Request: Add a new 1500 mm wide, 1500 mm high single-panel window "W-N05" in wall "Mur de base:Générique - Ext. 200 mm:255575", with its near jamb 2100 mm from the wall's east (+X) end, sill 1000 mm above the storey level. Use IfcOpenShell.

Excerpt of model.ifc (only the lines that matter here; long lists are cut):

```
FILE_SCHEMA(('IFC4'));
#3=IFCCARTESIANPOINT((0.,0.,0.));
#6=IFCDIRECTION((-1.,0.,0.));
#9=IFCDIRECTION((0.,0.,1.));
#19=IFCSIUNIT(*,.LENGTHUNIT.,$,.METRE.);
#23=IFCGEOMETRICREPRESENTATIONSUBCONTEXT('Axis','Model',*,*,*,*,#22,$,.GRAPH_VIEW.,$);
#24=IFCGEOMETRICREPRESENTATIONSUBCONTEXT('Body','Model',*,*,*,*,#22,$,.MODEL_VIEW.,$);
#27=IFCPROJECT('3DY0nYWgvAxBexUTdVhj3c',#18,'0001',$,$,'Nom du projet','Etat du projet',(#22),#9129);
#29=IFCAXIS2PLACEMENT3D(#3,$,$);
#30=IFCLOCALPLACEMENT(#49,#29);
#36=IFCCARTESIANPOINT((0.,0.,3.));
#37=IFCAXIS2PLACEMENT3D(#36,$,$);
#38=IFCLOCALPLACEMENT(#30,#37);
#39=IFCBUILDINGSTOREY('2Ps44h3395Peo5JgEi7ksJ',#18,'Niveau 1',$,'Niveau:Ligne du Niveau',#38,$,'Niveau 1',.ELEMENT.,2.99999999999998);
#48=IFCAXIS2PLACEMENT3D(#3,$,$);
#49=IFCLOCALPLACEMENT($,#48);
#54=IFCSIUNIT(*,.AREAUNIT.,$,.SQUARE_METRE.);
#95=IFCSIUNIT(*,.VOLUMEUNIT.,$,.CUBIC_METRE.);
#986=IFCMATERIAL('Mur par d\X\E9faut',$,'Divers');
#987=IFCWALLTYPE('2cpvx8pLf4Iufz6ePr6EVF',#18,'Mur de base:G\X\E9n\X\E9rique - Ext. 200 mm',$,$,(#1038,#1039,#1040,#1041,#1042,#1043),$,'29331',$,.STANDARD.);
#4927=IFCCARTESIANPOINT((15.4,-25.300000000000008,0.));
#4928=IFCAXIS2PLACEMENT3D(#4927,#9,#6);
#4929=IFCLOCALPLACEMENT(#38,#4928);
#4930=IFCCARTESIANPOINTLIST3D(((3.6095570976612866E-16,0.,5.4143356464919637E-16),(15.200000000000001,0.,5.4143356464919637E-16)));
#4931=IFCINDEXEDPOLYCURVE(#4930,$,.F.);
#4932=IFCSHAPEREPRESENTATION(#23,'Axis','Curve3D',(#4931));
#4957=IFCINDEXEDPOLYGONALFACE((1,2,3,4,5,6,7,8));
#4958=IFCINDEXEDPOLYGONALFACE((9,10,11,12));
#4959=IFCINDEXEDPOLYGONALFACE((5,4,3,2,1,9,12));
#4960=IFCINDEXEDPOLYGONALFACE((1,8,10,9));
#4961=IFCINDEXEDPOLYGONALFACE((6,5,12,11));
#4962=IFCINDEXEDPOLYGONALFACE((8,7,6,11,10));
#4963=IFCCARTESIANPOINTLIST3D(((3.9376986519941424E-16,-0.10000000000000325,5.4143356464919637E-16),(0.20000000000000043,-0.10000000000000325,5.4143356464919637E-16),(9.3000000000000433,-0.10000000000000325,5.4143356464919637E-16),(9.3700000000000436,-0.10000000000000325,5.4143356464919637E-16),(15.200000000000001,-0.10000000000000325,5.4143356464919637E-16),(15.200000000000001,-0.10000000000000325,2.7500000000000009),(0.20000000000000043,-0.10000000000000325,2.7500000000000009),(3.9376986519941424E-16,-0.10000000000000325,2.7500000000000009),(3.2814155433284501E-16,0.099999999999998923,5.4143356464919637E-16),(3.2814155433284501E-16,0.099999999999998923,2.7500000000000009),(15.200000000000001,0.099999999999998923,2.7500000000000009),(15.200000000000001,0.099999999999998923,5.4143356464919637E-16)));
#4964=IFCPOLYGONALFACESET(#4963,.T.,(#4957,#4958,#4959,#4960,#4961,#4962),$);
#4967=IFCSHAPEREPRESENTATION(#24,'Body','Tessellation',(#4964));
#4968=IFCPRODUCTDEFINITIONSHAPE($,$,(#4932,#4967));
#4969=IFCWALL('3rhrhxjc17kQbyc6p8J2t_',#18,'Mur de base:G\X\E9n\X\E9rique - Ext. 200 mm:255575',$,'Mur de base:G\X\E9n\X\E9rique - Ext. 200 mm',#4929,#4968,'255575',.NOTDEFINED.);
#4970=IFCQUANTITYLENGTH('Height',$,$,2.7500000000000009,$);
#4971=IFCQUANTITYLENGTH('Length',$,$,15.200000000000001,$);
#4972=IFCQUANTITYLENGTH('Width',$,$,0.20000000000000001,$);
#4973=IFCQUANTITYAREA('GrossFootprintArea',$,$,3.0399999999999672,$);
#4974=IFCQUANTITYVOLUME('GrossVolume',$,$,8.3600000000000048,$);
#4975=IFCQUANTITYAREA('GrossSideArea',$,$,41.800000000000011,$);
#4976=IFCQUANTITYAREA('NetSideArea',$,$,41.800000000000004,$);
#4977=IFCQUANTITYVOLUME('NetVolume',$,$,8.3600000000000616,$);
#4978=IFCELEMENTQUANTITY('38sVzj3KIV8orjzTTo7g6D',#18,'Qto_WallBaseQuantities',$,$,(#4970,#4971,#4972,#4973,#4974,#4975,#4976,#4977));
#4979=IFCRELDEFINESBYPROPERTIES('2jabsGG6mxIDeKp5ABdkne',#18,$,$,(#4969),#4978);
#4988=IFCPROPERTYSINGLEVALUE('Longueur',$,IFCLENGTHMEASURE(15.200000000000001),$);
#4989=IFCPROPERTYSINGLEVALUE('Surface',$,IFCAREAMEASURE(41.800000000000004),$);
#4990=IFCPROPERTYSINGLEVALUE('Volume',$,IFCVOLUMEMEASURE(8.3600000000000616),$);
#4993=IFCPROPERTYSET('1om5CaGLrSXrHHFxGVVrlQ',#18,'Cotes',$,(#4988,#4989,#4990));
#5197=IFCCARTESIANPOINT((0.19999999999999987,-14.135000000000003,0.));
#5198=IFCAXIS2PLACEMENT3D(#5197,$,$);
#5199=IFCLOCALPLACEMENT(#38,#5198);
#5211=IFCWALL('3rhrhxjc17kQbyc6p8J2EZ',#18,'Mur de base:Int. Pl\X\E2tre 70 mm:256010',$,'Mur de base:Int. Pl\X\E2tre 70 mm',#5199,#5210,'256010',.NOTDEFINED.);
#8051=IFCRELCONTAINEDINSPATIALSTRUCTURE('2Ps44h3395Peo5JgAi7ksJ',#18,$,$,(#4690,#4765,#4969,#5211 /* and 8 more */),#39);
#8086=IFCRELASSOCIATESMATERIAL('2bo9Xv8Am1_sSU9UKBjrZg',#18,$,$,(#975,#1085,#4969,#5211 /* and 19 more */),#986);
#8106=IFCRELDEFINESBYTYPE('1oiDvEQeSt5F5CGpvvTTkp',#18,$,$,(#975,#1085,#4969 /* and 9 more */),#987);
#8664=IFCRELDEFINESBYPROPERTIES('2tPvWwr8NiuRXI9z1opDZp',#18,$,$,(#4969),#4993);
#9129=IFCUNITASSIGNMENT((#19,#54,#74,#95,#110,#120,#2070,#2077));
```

```python
import numpy as np
import ifcopenshell
import ifcopenshell.api.feature
import ifcopenshell.api.geometry
import ifcopenshell.api.pset
import ifcopenshell.api.root
import ifcopenshell.api.spatial
import ifcopenshell.geom
import ifcopenshell.util.element
import ifcopenshell.util.placement
import ifcopenshell.util.representation
import ifcopenshell.util.shape
import ifcopenshell.util.unit

model = ifcopenshell.open("model.ifc")
unit_scale = ifcopenshell.util.unit.calculate_unit_scale(model)
area_scale = ifcopenshell.util.unit.calculate_unit_scale(model, "AREAUNIT")
volume_scale = ifcopenshell.util.unit.calculate_unit_scale(model, "VOLUMEUNIT")
settings = ifcopenshell.geom.settings()


def volume(element):
    """Net volume in cubic metres, openings subtracted."""
    shape = ifcopenshell.geom.create_shape(settings, element)
    return ifcopenshell.util.shape.get_volume(shape.geometry)


wall = model.by_id(4969)
storey = ifcopenshell.util.element.get_container(wall, ifc_class="IfcBuildingStorey")
context = ifcopenshell.util.representation.get_context(model, "Model", "Body", "MODEL_VIEW")
before = volume(wall)

width, height, from_end, sill = 1.5, 1.5, 2.1, 1  # metres

# The wall runs along its own X axis, and the end named is its -X end.
wall_shape = ifcopenshell.geom.create_shape(settings, wall)
x, y, z = ifcopenshell.util.shape.get_vertices(wall_shape.geometry).T
start = x.min() + from_end
face, thickness = float(y.min()), float(y.max() - y.min())
wall_matrix = ifcopenshell.util.placement.get_local_placement(wall.ObjectPlacement)
level = ifcopenshell.util.placement.get_local_placement(storey.ObjectPlacement)[2, 3]


def in_wall(x, y):
    """Placement at x, y metres in the wall's axes, at sill height."""
    matrix = wall_matrix.copy()
    matrix[:, 3] = wall_matrix @ np.array([x / unit_scale, y / unit_scale, 0.0, 1.0])
    matrix[2, 3] = level + sill / unit_scale
    return matrix


# Opening: a box that overshoots both wall faces by 50 mm.
opening = ifcopenshell.api.root.create_entity(model, ifc_class="IfcOpeningElement", predefined_type="OPENING")
box = ifcopenshell.api.geometry.add_wall_representation(
    model, context=context, length=width, height=height, thickness=thickness + 0.1
)
ifcopenshell.api.geometry.assign_representation(model, product=opening, representation=box)
ifcopenshell.api.geometry.edit_object_placement(model, product=opening, matrix=in_wall(start, face - 0.05), is_si=False)
ifcopenshell.api.feature.add_feature(model, feature=opening, element=wall)

window = ifcopenshell.api.root.create_entity(model, ifc_class="IfcWindow", name="W-N05", predefined_type="WINDOW")
window.OverallWidth, window.OverallHeight = width / unit_scale, height / unit_scale
window.PartitioningType = "SINGLE_PANEL"
body = ifcopenshell.api.geometry.add_window_representation(
    model,
    context=context,
    overall_width=window.OverallWidth,
    overall_height=window.OverallHeight,
    partition_type="SINGLE_PANEL",
)
ifcopenshell.api.geometry.assign_representation(model, product=window, representation=body)
ifcopenshell.api.spatial.assign_container(model, products=[window], relating_structure=storey)
ifcopenshell.api.feature.add_filling(model, opening=opening, element=window)

# Centre the window in the wall's thickness.
ifcopenshell.api.geometry.edit_object_placement(model, product=window, matrix=in_wall(start, face), is_si=False)
window_shape = ifcopenshell.geom.create_shape(settings, window)
depth = ifcopenshell.util.shape.get_vertices(window_shape.geometry)[:, 1]
offset = face + thickness / 2 - (depth.min() + depth.max()) / 2
ifcopenshell.api.geometry.edit_object_placement(model, product=window, matrix=in_wall(start, offset), is_si=False)

after = volume(wall)

# Update the wall's stored quantities.
qto = model.by_id(ifcopenshell.util.element.get_pset(wall, "Qto_WallBaseQuantities", should_inherit=False)["id"])
ifcopenshell.api.pset.edit_qto(model, qto=qto, properties={
    "NetSideArea": after / thickness / area_scale,
    "NetVolume": after / volume_scale,
})
pset = model.by_id(ifcopenshell.util.element.get_pset(wall, "Cotes", should_inherit=False)["id"])
ifcopenshell.api.pset.edit_pset(model, pset=pset, properties={
    "Surface": model.create_entity("IfcAreaMeasure", after / thickness / area_scale),
    "Volume": model.create_entity("IfcVolumeMeasure", after / volume_scale),
})

print(f"wall volume {before:.3f} -> {after:.3f} m3")

model.write("model_v2.ifc")
```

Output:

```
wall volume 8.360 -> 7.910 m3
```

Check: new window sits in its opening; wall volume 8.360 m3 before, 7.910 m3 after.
